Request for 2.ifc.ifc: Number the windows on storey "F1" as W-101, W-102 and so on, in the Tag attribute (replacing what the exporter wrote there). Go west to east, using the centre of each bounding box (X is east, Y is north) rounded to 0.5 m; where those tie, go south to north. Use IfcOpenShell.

First a look at what the model holds.

```python
import ifcopenshell
import ifcopenshell.util.element
import ifcopenshell.util.placement

model = ifcopenshell.open("2.ifc.ifc")
print(model.schema)
storey = next(s for s in model.by_type("IfcBuildingStorey") if s.Name == "F1")
windows = [e for e in ifcopenshell.util.element.get_decomposition(storey) if e.is_a("IfcWindow")]
for e in sorted(windows, key=lambda e: e.id()):
    origin = ifcopenshell.util.placement.get_local_placement(e.ObjectPlacement)[:3, 3]
    print(e.id(), e.Tag, e.Name, origin.round(2) + 0.0, sep=" | ")
```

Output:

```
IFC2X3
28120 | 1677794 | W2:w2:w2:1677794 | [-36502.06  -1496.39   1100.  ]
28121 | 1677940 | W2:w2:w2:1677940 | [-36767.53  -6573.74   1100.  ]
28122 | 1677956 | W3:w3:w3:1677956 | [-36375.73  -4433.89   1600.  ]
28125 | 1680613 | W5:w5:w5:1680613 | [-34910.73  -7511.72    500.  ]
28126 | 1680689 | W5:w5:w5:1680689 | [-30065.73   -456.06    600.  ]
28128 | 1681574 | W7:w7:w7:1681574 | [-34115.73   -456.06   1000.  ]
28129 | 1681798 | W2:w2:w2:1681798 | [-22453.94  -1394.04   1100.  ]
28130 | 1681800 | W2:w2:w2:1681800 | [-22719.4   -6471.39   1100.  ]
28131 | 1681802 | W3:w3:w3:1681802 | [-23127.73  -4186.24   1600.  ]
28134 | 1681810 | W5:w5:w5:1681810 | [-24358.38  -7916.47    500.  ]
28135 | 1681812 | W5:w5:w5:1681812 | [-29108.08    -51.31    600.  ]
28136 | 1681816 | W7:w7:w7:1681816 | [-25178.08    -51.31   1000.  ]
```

```python
import ifcopenshell
import ifcopenshell.geom
import ifcopenshell.util.element
import ifcopenshell.util.shape

model = ifcopenshell.open("2.ifc.ifc")
settings = ifcopenshell.geom.settings()
settings.set("use-world-coords", True)


def centre(element):
    shape = ifcopenshell.geom.create_shape(settings, element)
    return ifcopenshell.util.shape.get_bbox_centroid(shape.geometry)


storey = next(s for s in model.by_type("IfcBuildingStorey") if s.Name == "F1")
windows = [e for e in ifcopenshell.util.element.get_decomposition(storey) if e.is_a("IfcWindow")]

# Insertion points can sit at a corner or the storey origin, so sort by the geometry (in metres).
centres = {e: centre(e) for e in windows}
windows.sort(key=lambda e: (round(centres[e][0] / 0.5), centres[e][1]))

for i, e in enumerate(windows, start=1):
    number = f"W-1{i:02d}"
    e.Tag = number
    print(e.id(), number)

model.write("2.ifc_rev.ifc")
```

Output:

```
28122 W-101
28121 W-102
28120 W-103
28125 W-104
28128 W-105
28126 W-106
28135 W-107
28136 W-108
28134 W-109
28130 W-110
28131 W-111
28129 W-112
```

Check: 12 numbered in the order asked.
